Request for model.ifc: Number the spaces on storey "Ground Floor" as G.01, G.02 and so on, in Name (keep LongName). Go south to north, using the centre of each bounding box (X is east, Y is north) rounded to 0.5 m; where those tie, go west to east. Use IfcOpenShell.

First a look at what the model holds.

```python
import ifcopenshell
import ifcopenshell.util.element
import ifcopenshell.util.placement

model = ifcopenshell.open("model.ifc")
print(model.schema)
storey = next(s for s in model.by_type("IfcBuildingStorey") if s.Name == "Ground Floor")
spaces = [e for e in ifcopenshell.util.element.get_decomposition(storey) if e.is_a("IfcSpace")]
for e in sorted(spaces, key=lambda e: e.id()):
    origin = ifcopenshell.util.placement.get_local_placement(e.ObjectPlacement)[:3, 3]
    print(e.id(), e.Name, e.LongName, origin.round(2) + 0.0, sep=" | ")
```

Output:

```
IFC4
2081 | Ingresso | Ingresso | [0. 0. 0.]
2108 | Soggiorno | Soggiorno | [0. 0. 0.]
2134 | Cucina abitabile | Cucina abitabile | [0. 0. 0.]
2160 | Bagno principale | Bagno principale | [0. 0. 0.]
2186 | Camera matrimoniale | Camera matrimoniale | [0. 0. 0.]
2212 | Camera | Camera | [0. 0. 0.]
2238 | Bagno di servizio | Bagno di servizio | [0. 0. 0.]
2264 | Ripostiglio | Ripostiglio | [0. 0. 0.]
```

```python
import ifcopenshell
import ifcopenshell.geom
import ifcopenshell.util.element
import ifcopenshell.util.shape

model = ifcopenshell.open("model.ifc")
settings = ifcopenshell.geom.settings()
settings.set("use-world-coords", True)


def centre(element):
    shape = ifcopenshell.geom.create_shape(settings, element)
    return ifcopenshell.util.shape.get_bbox_centroid(shape.geometry)


storey = next(s for s in model.by_type("IfcBuildingStorey") if s.Name == "Ground Floor")
spaces = [e for e in ifcopenshell.util.element.get_decomposition(storey) if e.is_a("IfcSpace")]

# Insertion points can sit at a corner or the storey origin, so sort by the geometry (in metres).
centres = {e: centre(e) for e in spaces}
spaces.sort(key=lambda e: (round(centres[e][1] / 0.5), centres[e][0]))

for i, e in enumerate(spaces, start=1):
    number = f"G.{i:02d}"
    e.Name = number
    print(e.id(), number)

model.write("model-out.ifc")
```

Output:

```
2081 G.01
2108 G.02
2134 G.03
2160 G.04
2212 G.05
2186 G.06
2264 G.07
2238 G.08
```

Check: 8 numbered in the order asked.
